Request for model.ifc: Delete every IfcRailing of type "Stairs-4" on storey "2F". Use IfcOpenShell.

First a look at what the model holds.

```python
import ifcopenshell
import ifcopenshell.util.element

model = ifcopenshell.open("model.ifc")
print(model.schema)
storey = next(s for s in model.by_type("IfcBuildingStorey") if s.Name == "2F")
railings = [e for e in ifcopenshell.util.element.get_decomposition(storey) if e.is_a("IfcRailing")]
seen = {}
for e in railings:
    element_type = ifcopenshell.util.element.get_type(e)
    name = element_type.Name if element_type not in (None, e) else None
    seen[name] = seen.get(name, 0) + 1
for name, count in sorted(seen.items(), key=str):
    print(count, "x", name)
```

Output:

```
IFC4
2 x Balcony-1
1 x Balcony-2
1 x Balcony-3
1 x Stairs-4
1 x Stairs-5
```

```python
import ifcopenshell
import ifcopenshell.api.root
import ifcopenshell.util.element

model = ifcopenshell.open("model.ifc")

storey = next(s for s in model.by_type("IfcBuildingStorey") if s.Name == "2F")
railings = [e for e in ifcopenshell.util.element.get_decomposition(storey) if e.is_a("IfcRailing")]
targets = [e for e in railings if (t := ifcopenshell.util.element.get_type(e)) not in (None, e) and t.Name == "Stairs-4"]

for e in targets:
    ifcopenshell.api.root.remove_product(model, product=e)
print(len(targets), "removed")

model.write("model_updated.ifc")
```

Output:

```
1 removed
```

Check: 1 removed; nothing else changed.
